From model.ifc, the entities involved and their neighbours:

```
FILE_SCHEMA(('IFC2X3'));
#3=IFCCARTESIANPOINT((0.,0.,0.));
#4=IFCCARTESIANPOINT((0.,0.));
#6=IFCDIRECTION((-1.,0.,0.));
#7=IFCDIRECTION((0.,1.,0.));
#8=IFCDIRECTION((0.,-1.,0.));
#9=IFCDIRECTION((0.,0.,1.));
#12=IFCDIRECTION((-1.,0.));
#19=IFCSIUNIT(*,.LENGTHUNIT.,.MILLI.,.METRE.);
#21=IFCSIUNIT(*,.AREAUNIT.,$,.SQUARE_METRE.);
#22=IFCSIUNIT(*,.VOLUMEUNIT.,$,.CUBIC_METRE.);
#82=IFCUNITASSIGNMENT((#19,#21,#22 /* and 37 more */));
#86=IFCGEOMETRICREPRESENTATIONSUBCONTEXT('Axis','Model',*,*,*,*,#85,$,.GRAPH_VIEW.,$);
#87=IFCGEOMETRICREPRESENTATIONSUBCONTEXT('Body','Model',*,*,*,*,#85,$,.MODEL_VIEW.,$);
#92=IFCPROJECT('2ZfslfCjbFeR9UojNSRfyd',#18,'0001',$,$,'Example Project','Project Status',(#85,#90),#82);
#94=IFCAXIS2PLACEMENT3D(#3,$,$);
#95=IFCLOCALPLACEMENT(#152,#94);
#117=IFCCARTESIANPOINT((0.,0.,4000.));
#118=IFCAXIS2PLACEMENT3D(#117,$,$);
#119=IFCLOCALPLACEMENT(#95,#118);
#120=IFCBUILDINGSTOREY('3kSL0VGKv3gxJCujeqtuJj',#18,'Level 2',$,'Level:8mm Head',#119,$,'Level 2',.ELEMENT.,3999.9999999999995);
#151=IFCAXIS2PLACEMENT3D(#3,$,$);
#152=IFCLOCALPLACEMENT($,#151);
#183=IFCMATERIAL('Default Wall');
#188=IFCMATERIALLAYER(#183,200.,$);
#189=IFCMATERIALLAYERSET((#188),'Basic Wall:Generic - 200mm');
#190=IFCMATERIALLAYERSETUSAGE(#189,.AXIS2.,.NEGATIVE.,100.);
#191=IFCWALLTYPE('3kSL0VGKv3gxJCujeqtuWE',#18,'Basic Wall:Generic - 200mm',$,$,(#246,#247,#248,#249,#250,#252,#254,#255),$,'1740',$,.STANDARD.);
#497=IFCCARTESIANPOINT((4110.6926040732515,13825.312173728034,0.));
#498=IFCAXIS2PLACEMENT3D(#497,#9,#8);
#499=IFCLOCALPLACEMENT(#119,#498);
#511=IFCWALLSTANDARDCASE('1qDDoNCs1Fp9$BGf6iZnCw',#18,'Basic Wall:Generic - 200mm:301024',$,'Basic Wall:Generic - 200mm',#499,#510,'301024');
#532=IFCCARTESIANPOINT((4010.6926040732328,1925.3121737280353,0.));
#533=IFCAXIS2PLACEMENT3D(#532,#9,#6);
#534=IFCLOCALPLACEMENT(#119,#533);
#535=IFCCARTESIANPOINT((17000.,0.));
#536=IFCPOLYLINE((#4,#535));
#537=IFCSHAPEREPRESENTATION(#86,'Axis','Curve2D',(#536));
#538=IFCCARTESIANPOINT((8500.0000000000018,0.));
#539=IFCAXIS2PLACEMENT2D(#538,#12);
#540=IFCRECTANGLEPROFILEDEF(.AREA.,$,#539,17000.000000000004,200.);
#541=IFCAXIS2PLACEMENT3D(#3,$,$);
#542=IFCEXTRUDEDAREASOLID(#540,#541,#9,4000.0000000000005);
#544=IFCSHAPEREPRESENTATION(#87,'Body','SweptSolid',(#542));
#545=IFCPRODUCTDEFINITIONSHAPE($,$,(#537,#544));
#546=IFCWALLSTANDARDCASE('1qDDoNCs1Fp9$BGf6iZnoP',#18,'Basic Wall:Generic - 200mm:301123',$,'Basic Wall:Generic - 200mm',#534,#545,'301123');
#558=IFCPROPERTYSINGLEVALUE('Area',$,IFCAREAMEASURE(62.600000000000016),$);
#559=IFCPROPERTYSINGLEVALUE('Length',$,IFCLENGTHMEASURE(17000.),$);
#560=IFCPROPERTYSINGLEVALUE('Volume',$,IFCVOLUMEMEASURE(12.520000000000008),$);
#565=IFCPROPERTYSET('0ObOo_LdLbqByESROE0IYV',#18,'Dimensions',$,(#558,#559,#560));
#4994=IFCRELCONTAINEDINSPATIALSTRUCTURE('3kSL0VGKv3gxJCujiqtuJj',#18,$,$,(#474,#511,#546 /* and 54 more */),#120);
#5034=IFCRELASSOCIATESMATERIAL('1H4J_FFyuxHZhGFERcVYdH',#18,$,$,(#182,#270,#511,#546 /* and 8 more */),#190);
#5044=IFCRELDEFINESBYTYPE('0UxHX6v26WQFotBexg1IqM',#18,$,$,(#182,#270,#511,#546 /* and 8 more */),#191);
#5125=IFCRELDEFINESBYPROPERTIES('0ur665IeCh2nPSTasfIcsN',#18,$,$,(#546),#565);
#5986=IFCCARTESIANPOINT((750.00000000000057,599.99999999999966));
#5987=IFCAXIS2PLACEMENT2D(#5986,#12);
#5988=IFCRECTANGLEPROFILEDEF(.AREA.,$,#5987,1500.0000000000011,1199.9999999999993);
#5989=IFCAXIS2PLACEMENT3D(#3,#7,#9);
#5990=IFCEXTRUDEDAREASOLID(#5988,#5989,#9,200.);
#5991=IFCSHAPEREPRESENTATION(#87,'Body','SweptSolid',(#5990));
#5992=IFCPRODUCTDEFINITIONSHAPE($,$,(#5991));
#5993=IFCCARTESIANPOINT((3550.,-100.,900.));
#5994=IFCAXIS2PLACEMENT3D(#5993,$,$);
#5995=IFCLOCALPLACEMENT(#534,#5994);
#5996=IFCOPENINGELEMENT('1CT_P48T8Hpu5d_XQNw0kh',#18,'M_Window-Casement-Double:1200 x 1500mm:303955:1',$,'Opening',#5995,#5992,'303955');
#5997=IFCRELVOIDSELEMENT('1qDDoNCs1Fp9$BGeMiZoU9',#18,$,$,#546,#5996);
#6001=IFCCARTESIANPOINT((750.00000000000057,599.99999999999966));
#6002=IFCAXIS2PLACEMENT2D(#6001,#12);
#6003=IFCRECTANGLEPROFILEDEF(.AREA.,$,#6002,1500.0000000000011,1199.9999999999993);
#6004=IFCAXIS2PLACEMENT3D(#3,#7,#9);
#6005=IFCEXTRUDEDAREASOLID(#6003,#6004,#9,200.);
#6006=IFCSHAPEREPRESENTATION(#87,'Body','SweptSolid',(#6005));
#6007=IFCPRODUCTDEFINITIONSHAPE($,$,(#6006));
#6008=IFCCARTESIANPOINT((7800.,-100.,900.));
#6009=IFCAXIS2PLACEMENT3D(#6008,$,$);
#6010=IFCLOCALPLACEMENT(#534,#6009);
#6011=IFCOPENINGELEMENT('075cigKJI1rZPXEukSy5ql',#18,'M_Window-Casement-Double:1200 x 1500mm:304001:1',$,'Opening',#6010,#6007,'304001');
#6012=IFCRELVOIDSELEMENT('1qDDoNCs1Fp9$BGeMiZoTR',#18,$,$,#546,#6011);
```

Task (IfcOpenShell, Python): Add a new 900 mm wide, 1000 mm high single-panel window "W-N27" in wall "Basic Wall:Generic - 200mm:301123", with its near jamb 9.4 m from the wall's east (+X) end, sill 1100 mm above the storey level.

```python
import numpy as np
import ifcopenshell
import ifcopenshell.api.feature
import ifcopenshell.api.geometry
import ifcopenshell.api.pset
import ifcopenshell.api.root
import ifcopenshell.api.spatial
import ifcopenshell.api.type
import ifcopenshell.geom
import ifcopenshell.util.element
import ifcopenshell.util.placement
import ifcopenshell.util.representation
import ifcopenshell.util.shape
import ifcopenshell.util.unit

model = ifcopenshell.open("model.ifc")
unit_scale = ifcopenshell.util.unit.calculate_unit_scale(model)
area_scale = ifcopenshell.util.unit.calculate_unit_scale(model, "AREAUNIT")
volume_scale = ifcopenshell.util.unit.calculate_unit_scale(model, "VOLUMEUNIT")
settings = ifcopenshell.geom.settings()


def volume(element):
    """Net volume in cubic metres, openings subtracted."""
    shape = ifcopenshell.geom.create_shape(settings, element)
    return ifcopenshell.util.shape.get_volume(shape.geometry)


wall = model.by_guid("1qDDoNCs1Fp9$BGf6iZnoP")
storey = ifcopenshell.util.element.get_container(wall, ifc_class="IfcBuildingStorey")
context = ifcopenshell.util.representation.get_context(model, "Model", "Body", "MODEL_VIEW")
before = volume(wall)

width, height, from_end, sill = 0.9, 1, 9.4, 1.1  # metres

# The wall runs along its own X axis, and the end named is its -X end.
wall_shape = ifcopenshell.geom.create_shape(settings, wall)
x, y, z = ifcopenshell.util.shape.get_vertices(wall_shape.geometry).T
start = x.min() + from_end
face, thickness = float(y.min()), float(y.max() - y.min())
wall_matrix = ifcopenshell.util.placement.get_local_placement(wall.ObjectPlacement)
level = ifcopenshell.util.placement.get_local_placement(storey.ObjectPlacement)[2, 3]


def in_wall(x, y):
    """Placement at x, y metres in the wall's axes, at sill height."""
    matrix = wall_matrix.copy()
    matrix[:, 3] = wall_matrix @ np.array([x / unit_scale, y / unit_scale, 0.0, 1.0])
    matrix[2, 3] = level + sill / unit_scale
    return matrix


# Opening: a box that overshoots both wall faces by 50 mm.
opening = ifcopenshell.api.root.create_entity(model, ifc_class="IfcOpeningElement")
box = ifcopenshell.api.geometry.add_wall_representation(
    model, context=context, length=width, height=height, thickness=thickness + 0.1
)
ifcopenshell.api.geometry.assign_representation(model, product=opening, representation=box)
ifcopenshell.api.geometry.edit_object_placement(model, product=opening, matrix=in_wall(start, face - 0.05), is_si=False)
ifcopenshell.api.feature.add_feature(model, feature=opening, element=wall)

window = ifcopenshell.api.root.create_entity(model, ifc_class="IfcWindow", name="W-N27")
window.OverallWidth, window.OverallHeight = width / unit_scale, height / unit_scale
body = ifcopenshell.api.geometry.add_window_representation(
    model,
    context=context,
    overall_width=window.OverallWidth,
    overall_height=window.OverallHeight,
    partition_type="SINGLE_PANEL",
)
ifcopenshell.api.geometry.assign_representation(model, product=window, representation=body)
ifcopenshell.api.spatial.assign_container(model, products=[window], relating_structure=storey)
fills = ifcopenshell.api.feature.add_filling(model, opening=opening, element=window)
fills.OwnerHistory = window.OwnerHistory  # required in IFC2X3

# IFC2X3 keeps the operation on the window style.
style = ifcopenshell.api.root.create_entity(model, ifc_class="IfcWindowStyle", name="W-N27")
style.OperationType, style.ConstructionType = "SINGLE_PANEL", "NOTDEFINED"
style.ParameterTakesPrecedence = style.Sizeable = False
ifcopenshell.api.type.assign_type(model, related_objects=[window], relating_type=style)

# Centre the window in the wall's thickness.
ifcopenshell.api.geometry.edit_object_placement(model, product=window, matrix=in_wall(start, face), is_si=False)
window_shape = ifcopenshell.geom.create_shape(settings, window)
depth = ifcopenshell.util.shape.get_vertices(window_shape.geometry)[:, 1]
offset = face + thickness / 2 - (depth.min() + depth.max()) / 2
ifcopenshell.api.geometry.edit_object_placement(model, product=window, matrix=in_wall(start, offset), is_si=False)

after = volume(wall)

# Update the wall's stored quantities.
pset = model.by_id(ifcopenshell.util.element.get_pset(wall, "Dimensions", should_inherit=False)["id"])
ifcopenshell.api.pset.edit_pset(model, pset=pset, properties={
    "Area": model.create_entity("IfcAreaMeasure", after / thickness / area_scale),
    "Volume": model.create_entity("IfcVolumeMeasure", after / volume_scale),
})

print(f"wall volume {before:.3f} -> {after:.3f} m3")

model.write("model_rev.ifc")
```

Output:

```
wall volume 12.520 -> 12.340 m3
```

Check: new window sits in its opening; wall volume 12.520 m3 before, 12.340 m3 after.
